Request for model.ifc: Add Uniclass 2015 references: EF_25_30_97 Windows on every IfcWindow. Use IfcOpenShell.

First a look at what the model holds.

```python
import ifcopenshell

model = ifcopenshell.open("model.ifc")
print(model.schema)
print("classifications:", [c.Name for c in model.by_type("IfcClassification")])
for ifc_class in ("IfcDoor", "IfcRoof", "IfcStair", "IfcWall", "IfcWindow"):
    print(ifc_class, len(model.by_type(ifc_class)))
```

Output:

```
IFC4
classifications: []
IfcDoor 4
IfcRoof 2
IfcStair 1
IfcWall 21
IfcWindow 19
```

```python
import ifcopenshell
import ifcopenshell.api.classification

model = ifcopenshell.open("model.ifc")

system = ifcopenshell.api.classification.add_classification(model, classification="Uniclass 2015")

codes = {
    "IfcWindow": ("EF_25_30_97", "Windows"),
}
for ifc_class, (code, name) in codes.items():
    products = model.by_type(ifc_class)
    ifcopenshell.api.classification.add_reference(
        model, products=products, classification=system, identification=code, name=name
    )
    print(code, len(products))

model.write("model_updated.ifc")
```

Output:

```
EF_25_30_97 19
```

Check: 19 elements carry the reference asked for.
